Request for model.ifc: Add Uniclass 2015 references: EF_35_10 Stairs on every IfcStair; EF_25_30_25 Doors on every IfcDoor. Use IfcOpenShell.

First a look at what the model holds.

```python
import ifcopenshell

model = ifcopenshell.open("model.ifc")
print(model.schema)
print("classifications:", [c.Name for c in model.by_type("IfcClassification")])
for ifc_class in ("IfcDoor", "IfcRoof", "IfcStair", "IfcWall", "IfcWindow"):
    print(ifc_class, len(model.by_type(ifc_class)))
```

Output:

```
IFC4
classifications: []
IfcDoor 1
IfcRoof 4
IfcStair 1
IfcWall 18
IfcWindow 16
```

```python
import ifcopenshell
import ifcopenshell.api.classification

model = ifcopenshell.open("model.ifc")

system = ifcopenshell.api.classification.add_classification(model, classification="Uniclass 2015")

codes = {
    "IfcStair": ("EF_35_10", "Stairs"),
    "IfcDoor": ("EF_25_30_25", "Doors"),
}
for ifc_class, (code, name) in codes.items():
    products = model.by_type(ifc_class)
    ifcopenshell.api.classification.add_reference(
        model, products=products, classification=system, identification=code, name=name
    )
    print(code, len(products))

model.write("model_rev.ifc")
```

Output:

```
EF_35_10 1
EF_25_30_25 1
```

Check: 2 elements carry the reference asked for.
